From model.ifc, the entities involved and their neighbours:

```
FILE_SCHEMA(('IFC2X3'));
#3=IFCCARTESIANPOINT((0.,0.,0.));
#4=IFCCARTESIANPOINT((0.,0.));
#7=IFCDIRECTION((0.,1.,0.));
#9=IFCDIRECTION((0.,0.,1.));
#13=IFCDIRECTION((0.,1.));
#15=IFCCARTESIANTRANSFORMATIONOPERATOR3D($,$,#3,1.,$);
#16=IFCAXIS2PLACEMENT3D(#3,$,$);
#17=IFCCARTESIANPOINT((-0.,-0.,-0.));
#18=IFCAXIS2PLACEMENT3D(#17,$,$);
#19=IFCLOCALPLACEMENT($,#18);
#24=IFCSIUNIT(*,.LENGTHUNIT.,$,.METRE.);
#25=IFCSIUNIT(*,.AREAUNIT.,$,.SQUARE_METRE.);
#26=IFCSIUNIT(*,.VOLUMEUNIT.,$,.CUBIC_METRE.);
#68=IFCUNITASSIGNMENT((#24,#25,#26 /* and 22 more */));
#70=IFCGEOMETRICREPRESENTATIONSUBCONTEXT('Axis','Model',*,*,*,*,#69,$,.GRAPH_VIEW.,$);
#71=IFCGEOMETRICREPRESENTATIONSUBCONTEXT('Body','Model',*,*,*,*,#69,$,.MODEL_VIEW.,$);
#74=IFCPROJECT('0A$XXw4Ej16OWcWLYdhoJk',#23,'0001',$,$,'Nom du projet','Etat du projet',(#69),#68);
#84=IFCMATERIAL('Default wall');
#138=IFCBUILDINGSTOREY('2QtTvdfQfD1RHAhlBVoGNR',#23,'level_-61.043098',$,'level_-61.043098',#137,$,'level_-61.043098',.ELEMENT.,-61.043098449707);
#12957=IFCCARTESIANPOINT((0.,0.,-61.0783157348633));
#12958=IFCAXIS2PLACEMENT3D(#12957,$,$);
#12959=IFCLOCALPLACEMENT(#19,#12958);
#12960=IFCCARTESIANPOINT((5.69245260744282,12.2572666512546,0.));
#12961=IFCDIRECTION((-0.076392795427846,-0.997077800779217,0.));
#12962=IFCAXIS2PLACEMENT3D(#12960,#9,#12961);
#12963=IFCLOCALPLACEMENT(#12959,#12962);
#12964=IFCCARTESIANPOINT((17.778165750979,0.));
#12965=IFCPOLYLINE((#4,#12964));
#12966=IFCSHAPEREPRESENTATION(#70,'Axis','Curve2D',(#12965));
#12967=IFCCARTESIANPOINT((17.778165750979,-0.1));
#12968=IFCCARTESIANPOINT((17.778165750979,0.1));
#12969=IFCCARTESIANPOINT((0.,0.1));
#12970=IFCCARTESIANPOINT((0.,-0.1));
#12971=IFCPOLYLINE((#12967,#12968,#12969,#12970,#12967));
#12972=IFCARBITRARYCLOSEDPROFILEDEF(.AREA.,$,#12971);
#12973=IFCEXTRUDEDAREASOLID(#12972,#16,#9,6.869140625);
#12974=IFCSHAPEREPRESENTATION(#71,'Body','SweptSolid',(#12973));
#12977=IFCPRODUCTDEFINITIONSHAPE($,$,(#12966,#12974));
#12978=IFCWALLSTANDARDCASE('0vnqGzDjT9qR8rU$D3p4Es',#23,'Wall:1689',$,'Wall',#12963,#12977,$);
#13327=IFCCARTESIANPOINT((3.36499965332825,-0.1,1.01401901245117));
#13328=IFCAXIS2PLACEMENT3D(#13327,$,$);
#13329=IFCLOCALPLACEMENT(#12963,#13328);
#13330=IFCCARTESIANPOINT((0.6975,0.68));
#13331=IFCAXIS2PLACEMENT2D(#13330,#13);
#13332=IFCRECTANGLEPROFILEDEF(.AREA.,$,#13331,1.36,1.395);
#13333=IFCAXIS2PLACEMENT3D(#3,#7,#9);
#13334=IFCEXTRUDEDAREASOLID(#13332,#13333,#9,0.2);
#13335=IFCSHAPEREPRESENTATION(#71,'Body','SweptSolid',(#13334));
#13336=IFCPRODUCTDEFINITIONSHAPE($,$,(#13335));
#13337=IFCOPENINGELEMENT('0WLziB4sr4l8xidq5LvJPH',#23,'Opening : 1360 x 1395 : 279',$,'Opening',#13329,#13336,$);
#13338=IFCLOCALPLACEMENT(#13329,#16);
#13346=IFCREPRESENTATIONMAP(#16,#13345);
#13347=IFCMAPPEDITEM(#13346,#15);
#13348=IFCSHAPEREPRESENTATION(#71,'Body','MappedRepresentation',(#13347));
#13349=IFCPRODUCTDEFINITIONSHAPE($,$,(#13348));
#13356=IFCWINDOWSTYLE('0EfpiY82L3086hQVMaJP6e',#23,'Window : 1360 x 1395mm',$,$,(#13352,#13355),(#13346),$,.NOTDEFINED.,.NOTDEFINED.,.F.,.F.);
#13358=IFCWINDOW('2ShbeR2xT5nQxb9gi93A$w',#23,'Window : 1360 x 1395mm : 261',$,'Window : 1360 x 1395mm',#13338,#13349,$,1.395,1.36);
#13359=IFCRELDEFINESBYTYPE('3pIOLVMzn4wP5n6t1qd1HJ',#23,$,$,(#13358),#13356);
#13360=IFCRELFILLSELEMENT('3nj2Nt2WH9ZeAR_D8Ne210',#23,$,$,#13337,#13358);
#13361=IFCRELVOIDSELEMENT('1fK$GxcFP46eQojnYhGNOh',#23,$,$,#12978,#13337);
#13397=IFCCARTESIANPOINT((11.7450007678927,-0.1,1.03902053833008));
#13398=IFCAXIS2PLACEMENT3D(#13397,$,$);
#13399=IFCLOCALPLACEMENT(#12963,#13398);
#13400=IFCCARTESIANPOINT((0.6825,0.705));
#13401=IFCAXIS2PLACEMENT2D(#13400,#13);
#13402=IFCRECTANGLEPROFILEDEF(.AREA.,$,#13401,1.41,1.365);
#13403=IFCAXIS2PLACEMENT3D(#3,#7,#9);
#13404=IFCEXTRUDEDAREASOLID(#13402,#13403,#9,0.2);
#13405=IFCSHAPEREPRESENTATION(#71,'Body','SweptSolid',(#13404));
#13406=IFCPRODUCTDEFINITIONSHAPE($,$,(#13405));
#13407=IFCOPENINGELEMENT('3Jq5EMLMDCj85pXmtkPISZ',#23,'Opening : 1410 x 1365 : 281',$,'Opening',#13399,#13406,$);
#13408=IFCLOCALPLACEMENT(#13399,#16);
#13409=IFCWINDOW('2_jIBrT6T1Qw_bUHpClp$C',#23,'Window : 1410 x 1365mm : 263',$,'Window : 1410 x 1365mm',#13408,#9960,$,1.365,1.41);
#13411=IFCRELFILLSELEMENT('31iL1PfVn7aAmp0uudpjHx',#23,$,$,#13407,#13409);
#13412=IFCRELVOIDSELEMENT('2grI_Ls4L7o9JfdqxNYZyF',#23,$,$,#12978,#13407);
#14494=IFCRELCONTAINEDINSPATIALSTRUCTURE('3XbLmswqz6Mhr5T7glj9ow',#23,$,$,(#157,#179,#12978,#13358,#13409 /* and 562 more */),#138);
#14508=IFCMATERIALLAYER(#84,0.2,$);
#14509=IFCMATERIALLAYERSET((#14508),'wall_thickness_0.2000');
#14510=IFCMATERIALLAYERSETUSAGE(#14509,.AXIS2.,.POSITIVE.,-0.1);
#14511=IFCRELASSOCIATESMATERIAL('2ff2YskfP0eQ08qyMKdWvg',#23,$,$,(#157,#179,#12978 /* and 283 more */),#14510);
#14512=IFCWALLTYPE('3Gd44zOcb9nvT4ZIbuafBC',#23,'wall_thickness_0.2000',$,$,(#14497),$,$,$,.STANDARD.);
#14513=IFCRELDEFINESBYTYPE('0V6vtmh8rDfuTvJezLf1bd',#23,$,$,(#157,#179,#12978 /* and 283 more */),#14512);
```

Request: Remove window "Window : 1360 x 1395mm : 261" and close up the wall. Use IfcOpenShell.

```python
import ifcopenshell
import ifcopenshell.api.feature
import ifcopenshell.api.root
import ifcopenshell.geom
import ifcopenshell.util.shape

model = ifcopenshell.open("model.ifc")
settings = ifcopenshell.geom.settings()


def volume(element):
    """Net volume in cubic metres, openings subtracted."""
    shape = ifcopenshell.geom.create_shape(settings, element)
    return ifcopenshell.util.shape.get_volume(shape.geometry)


window = model.by_guid("2ShbeR2xT5nQxb9gi93A$w")
opening = window.FillsVoids[0].RelatingOpeningElement
wall = opening.VoidsElements[0].RelatingBuildingElement
before = volume(wall)

ifcopenshell.api.root.remove_product(model, product=window)
ifcopenshell.api.feature.remove_feature(model, feature=opening)

after = volume(wall)

print(f"wall volume {before:.3f} -> {after:.3f} m3")

model.write("model_updated.ifc")
```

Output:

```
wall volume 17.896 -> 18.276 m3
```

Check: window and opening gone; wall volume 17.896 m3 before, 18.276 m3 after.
